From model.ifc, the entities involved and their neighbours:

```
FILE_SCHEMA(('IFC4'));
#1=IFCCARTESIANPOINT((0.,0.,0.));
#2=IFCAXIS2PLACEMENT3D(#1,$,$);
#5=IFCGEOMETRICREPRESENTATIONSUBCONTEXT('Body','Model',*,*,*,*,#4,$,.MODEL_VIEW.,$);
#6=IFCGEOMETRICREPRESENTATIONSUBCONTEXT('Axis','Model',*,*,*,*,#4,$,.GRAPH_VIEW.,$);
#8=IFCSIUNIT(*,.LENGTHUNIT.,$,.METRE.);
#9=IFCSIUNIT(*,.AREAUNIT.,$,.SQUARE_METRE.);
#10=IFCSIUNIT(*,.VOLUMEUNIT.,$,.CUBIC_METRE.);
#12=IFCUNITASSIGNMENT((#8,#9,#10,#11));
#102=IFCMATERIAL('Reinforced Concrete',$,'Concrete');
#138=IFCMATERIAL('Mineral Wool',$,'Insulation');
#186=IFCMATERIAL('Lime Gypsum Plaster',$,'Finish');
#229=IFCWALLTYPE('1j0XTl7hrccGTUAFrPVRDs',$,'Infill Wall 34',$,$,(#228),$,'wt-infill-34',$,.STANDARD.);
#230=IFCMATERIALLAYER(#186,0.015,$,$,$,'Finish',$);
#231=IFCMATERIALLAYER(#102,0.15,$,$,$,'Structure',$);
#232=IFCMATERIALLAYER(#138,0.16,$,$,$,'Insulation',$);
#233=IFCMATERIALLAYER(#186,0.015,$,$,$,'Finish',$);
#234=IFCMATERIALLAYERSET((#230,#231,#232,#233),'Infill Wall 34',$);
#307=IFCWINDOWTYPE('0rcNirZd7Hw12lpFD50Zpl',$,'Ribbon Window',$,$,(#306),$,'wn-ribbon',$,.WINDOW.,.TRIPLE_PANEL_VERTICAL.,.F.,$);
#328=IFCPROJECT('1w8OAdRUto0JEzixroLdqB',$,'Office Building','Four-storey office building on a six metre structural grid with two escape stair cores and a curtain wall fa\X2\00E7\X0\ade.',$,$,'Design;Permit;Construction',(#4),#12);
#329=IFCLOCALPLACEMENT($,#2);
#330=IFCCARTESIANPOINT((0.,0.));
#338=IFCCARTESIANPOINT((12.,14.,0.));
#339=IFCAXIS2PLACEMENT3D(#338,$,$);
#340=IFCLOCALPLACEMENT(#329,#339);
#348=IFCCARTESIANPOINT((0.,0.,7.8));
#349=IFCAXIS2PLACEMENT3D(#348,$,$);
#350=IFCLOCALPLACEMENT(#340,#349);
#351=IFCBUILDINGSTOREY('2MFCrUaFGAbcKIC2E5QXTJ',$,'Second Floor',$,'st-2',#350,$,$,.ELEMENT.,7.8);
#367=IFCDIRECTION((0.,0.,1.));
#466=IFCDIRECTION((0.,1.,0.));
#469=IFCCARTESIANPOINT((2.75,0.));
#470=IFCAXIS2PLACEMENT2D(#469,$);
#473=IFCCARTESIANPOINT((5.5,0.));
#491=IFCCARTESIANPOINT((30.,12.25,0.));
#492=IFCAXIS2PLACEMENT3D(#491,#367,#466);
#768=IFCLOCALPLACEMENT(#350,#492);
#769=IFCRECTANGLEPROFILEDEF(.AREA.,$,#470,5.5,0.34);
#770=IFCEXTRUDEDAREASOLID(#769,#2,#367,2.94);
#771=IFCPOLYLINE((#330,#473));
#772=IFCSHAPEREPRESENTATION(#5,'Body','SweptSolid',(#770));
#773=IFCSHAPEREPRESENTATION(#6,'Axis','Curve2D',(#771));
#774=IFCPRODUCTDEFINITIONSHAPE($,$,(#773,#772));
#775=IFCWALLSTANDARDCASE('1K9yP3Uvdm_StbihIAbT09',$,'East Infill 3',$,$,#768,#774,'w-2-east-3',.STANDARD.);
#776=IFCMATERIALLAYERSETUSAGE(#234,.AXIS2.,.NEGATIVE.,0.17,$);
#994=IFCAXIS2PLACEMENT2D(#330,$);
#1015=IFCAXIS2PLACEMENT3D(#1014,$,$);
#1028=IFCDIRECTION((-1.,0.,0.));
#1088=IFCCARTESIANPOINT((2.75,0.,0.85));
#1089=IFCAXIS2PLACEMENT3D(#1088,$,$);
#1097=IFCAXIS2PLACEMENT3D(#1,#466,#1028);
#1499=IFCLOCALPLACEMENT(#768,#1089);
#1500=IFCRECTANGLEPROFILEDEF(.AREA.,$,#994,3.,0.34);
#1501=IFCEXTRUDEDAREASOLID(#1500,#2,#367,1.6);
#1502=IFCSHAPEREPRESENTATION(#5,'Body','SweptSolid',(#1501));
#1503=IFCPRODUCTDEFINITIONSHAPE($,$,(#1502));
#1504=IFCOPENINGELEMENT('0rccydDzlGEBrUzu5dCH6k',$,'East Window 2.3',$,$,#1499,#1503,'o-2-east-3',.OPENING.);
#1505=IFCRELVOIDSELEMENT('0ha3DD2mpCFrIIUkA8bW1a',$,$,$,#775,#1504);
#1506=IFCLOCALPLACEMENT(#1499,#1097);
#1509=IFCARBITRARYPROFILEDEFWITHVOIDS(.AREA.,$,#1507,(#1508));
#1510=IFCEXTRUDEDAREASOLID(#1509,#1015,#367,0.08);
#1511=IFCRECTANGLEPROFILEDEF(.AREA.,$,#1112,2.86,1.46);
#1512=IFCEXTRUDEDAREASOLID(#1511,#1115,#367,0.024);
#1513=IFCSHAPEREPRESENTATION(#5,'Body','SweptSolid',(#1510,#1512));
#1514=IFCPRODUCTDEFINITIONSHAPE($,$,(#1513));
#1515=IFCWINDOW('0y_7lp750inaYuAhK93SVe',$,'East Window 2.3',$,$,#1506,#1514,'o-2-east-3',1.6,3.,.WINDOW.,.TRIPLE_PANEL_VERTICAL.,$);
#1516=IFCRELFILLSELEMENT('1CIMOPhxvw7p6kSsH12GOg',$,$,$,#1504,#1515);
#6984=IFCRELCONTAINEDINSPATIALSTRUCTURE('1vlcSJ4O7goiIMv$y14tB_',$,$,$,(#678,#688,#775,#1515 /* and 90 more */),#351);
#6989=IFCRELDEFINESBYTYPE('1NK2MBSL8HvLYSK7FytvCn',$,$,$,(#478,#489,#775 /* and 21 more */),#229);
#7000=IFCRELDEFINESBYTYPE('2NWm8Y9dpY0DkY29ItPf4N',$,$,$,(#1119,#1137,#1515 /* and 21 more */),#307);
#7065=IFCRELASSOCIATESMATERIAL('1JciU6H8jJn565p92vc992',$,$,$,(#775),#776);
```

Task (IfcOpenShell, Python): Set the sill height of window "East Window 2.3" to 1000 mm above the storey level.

```python
import numpy as np
import ifcopenshell
import ifcopenshell.api.geometry
import ifcopenshell.geom
import ifcopenshell.util.element
import ifcopenshell.util.placement
import ifcopenshell.util.shape
import ifcopenshell.util.unit

model = ifcopenshell.open("model.ifc")
unit_scale = ifcopenshell.util.unit.calculate_unit_scale(model)

window = model.by_id(1515)
opening = window.FillsVoids[0].RelatingOpeningElement
storey = ifcopenshell.util.element.get_container(window, ifc_class="IfcBuildingStorey")
level = ifcopenshell.util.placement.get_local_placement(storey.ObjectPlacement)[2, 3]

# The opening's origin need not be at the sill, so measure its lowest point.
shape = ifcopenshell.geom.create_shape(ifcopenshell.geom.settings(), opening)
bottom = ifcopenshell.util.shape.get_shape_bottom_elevation(shape, shape.geometry) / unit_scale
dz = level + 1 / unit_scale - bottom

shift = np.array([0.0, 0.0, dz])
# The window is placed relative to its opening, so it follows when the opening moves.
matrix = ifcopenshell.util.placement.get_local_placement(opening.ObjectPlacement)
matrix[:3, 3] += shift
ifcopenshell.api.geometry.edit_object_placement(
    model, product=opening, matrix=matrix, is_si=False, should_transform_children=True
)

print(f"moved by {dz * unit_scale:+.3f} m")

model.write("model_updated.ifc")
```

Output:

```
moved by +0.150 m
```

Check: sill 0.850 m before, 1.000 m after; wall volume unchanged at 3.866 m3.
